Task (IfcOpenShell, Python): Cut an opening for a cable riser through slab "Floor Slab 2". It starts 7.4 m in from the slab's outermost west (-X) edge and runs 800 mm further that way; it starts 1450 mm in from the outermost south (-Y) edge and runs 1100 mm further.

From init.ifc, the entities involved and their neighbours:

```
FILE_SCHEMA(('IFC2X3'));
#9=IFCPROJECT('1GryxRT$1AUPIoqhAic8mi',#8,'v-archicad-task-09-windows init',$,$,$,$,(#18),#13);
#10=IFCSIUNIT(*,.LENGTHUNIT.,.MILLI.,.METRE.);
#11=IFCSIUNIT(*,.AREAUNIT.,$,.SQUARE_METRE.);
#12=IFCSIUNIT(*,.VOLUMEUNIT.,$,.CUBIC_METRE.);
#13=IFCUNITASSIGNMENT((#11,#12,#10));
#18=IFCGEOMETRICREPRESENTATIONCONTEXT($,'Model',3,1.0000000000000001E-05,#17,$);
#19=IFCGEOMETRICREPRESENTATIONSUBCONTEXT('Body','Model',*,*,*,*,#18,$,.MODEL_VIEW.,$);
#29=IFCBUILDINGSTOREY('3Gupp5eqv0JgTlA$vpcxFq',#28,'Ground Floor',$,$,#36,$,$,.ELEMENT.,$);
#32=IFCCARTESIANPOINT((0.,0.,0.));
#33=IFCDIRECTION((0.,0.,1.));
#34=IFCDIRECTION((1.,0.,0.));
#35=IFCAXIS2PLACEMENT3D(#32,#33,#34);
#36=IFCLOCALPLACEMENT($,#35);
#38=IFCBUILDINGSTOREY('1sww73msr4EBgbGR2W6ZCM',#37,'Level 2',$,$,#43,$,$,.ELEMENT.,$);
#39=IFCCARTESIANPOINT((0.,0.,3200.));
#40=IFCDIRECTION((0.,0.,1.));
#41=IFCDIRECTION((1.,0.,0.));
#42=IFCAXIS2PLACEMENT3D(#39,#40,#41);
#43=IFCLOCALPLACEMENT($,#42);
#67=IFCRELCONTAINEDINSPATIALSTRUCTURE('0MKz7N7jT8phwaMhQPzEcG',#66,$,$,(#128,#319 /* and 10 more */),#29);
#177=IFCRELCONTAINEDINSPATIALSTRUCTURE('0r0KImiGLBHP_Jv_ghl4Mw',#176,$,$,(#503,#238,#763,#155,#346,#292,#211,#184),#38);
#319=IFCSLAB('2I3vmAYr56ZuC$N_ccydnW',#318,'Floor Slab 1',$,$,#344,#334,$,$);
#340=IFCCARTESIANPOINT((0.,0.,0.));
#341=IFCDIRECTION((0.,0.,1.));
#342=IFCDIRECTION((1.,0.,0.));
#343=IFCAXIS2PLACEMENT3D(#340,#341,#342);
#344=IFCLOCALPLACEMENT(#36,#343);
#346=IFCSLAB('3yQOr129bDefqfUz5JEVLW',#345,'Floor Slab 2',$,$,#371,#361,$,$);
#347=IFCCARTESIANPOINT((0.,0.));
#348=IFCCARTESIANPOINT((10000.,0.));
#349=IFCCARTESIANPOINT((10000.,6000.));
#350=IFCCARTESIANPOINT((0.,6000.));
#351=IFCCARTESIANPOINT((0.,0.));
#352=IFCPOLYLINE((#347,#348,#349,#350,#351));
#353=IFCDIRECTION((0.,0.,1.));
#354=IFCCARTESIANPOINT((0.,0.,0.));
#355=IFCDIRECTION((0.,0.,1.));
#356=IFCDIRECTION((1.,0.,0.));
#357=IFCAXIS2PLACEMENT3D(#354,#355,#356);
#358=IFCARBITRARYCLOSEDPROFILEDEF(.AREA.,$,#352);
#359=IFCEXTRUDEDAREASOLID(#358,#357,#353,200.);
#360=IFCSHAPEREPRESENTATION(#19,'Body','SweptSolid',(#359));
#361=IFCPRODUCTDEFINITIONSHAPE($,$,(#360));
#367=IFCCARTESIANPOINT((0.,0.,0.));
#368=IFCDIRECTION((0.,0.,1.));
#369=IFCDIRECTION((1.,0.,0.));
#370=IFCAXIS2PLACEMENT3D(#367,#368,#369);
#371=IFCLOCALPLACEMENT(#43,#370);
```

```python
import numpy as np
import ifcopenshell
import ifcopenshell.api.feature
import ifcopenshell.api.geometry
import ifcopenshell.api.root
import ifcopenshell.geom
import ifcopenshell.util.placement
import ifcopenshell.util.representation
import ifcopenshell.util.shape
import ifcopenshell.util.unit

model = ifcopenshell.open("init.ifc")
unit_scale = ifcopenshell.util.unit.calculate_unit_scale(model)
settings = ifcopenshell.geom.settings()


def volume(element):
    """Net volume in cubic metres, openings subtracted."""
    shape = ifcopenshell.geom.create_shape(settings, element)
    return ifcopenshell.util.shape.get_volume(shape.geometry)


slab = model.by_guid("3yQOr129bDefqfUz5JEVLW")
before = volume(slab)

# Extent in the slab's own axes, in metres. The edges named are its -X and -Y sides.
slab_shape = ifcopenshell.geom.create_shape(settings, slab)
vertices = ifcopenshell.util.shape.get_vertices(slab_shape.geometry)
x_min, y_min, bottom = vertices.min(axis=0)
top = vertices[:, 2].max()

opening = ifcopenshell.api.root.create_entity(model, ifc_class="IfcOpeningElement", name="Cable riser opening")
context = ifcopenshell.util.representation.get_context(model, "Model", "Body", "MODEL_VIEW")
width, depth = 0.8, 1.1
outline = [(0.0, 0.0), (width, 0.0), (width, depth), (0.0, depth), (0.0, 0.0)]
# Overshoot both faces by 50 mm so the cut is clean.
shape = ifcopenshell.api.geometry.add_slab_representation(
    model, context=context, depth=top - bottom + 0.1, polyline=outline
)
ifcopenshell.api.geometry.assign_representation(model, product=opening, representation=shape)

matrix = ifcopenshell.util.placement.get_local_placement(slab.ObjectPlacement)
matrix[:, 3] = matrix @ np.append(np.array([x_min + 7.4, y_min + 1.45, bottom - 0.05]) / unit_scale, 1.0)
ifcopenshell.api.geometry.edit_object_placement(model, product=opening, matrix=matrix, is_si=False)
ifcopenshell.api.feature.add_feature(model, feature=opening, element=slab)

after = volume(slab)

print(f"slab volume {before:.3f} -> {after:.3f} m3")

model.write("init-out.ifc")
```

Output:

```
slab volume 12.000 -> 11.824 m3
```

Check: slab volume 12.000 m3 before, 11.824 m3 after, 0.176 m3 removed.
